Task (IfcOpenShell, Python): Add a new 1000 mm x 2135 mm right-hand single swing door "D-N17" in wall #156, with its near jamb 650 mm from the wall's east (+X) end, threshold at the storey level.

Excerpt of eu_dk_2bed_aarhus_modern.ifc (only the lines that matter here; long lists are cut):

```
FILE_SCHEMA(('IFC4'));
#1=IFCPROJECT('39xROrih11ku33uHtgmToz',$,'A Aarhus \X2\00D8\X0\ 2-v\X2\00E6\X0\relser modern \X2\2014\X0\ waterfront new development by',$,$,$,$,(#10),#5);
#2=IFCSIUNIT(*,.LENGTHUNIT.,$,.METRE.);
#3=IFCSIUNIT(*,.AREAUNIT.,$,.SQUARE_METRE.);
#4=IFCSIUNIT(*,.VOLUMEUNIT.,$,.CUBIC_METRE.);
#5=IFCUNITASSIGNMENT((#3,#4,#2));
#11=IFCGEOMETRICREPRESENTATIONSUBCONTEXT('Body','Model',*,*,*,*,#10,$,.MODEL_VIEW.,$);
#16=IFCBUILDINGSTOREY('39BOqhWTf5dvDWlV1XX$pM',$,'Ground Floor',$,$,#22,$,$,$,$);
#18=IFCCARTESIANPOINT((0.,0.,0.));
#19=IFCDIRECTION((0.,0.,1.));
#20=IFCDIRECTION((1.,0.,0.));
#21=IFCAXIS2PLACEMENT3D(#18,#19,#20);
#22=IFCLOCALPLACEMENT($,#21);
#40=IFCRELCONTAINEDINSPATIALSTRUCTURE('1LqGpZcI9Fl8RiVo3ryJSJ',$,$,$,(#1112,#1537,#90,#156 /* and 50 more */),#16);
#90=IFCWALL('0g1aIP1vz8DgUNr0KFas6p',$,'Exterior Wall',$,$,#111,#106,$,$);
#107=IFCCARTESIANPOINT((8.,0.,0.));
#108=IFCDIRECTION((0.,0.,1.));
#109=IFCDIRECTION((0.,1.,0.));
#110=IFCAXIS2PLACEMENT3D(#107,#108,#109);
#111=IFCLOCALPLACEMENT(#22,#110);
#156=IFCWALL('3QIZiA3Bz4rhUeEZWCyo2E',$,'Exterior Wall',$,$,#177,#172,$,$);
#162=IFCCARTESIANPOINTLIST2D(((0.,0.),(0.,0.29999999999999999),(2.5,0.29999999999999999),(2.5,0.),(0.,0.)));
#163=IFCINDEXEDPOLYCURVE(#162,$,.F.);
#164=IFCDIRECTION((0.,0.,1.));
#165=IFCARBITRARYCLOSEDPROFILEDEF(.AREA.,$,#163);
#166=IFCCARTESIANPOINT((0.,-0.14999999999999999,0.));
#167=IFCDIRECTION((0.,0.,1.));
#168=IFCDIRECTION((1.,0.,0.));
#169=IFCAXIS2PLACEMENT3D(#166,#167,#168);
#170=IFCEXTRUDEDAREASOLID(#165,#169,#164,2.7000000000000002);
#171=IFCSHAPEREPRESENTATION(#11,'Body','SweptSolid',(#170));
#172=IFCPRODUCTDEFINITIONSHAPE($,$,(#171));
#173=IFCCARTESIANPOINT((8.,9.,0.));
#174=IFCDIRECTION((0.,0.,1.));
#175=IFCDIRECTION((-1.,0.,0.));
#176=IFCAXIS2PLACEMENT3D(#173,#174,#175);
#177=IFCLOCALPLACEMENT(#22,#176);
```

```python
import numpy as np
import ifcopenshell
import ifcopenshell.api.feature
import ifcopenshell.api.geometry
import ifcopenshell.api.root
import ifcopenshell.api.spatial
import ifcopenshell.geom
import ifcopenshell.util.element
import ifcopenshell.util.placement
import ifcopenshell.util.representation
import ifcopenshell.util.shape
import ifcopenshell.util.unit

model = ifcopenshell.open("eu_dk_2bed_aarhus_modern.ifc")
unit_scale = ifcopenshell.util.unit.calculate_unit_scale(model)
settings = ifcopenshell.geom.settings()


def volume(element):
    """Net volume in cubic metres, openings subtracted."""
    shape = ifcopenshell.geom.create_shape(settings, element)
    return ifcopenshell.util.shape.get_volume(shape.geometry)


wall = model.by_id(156)
storey = ifcopenshell.util.element.get_container(wall, ifc_class="IfcBuildingStorey")
context = ifcopenshell.util.representation.get_context(model, "Model", "Body", "MODEL_VIEW")
before = volume(wall)

width, height, from_end, sill = 1, 2.135, 0.65, 0.0  # metres

# The wall runs along its own X axis, and the end named is its -X end.
wall_shape = ifcopenshell.geom.create_shape(settings, wall)
x, y, z = ifcopenshell.util.shape.get_vertices(wall_shape.geometry).T
start = x.min() + from_end
face, thickness = float(y.min()), float(y.max() - y.min())
wall_matrix = ifcopenshell.util.placement.get_local_placement(wall.ObjectPlacement)
level = ifcopenshell.util.placement.get_local_placement(storey.ObjectPlacement)[2, 3]


def in_wall(x, y):
    """Placement at x, y metres in the wall's axes, at sill height."""
    matrix = wall_matrix.copy()
    matrix[:, 3] = wall_matrix @ np.array([x / unit_scale, y / unit_scale, 0.0, 1.0])
    matrix[2, 3] = level + sill / unit_scale
    return matrix


# Opening: a box that overshoots both wall faces by 50 mm.
opening = ifcopenshell.api.root.create_entity(model, ifc_class="IfcOpeningElement", predefined_type="OPENING")
box = ifcopenshell.api.geometry.add_wall_representation(
    model, context=context, length=width, height=height, thickness=thickness + 0.1
)
ifcopenshell.api.geometry.assign_representation(model, product=opening, representation=box)
ifcopenshell.api.geometry.edit_object_placement(model, product=opening, matrix=in_wall(start, face - 0.05), is_si=False)
ifcopenshell.api.feature.add_feature(model, feature=opening, element=wall)

door = ifcopenshell.api.root.create_entity(model, ifc_class="IfcDoor", name="D-N17", predefined_type="DOOR")
door.OverallWidth, door.OverallHeight = width / unit_scale, height / unit_scale
door.OperationType = "SINGLE_SWING_RIGHT"
body = ifcopenshell.api.geometry.add_door_representation(
    model,
    context=context,
    overall_width=door.OverallWidth,
    overall_height=door.OverallHeight,
    operation_type="SINGLE_SWING_RIGHT",
    lining_properties={"LiningDepth": thickness / unit_scale, "ThresholdDepth": thickness / unit_scale},
)
ifcopenshell.api.geometry.assign_representation(model, product=door, representation=body)
ifcopenshell.api.spatial.assign_container(model, products=[door], relating_structure=storey)
ifcopenshell.api.feature.add_filling(model, opening=opening, element=door)

# The lining spans the wall, so the door starts at the wall face.
ifcopenshell.api.geometry.edit_object_placement(model, product=door, matrix=in_wall(start, face), is_si=False)

after = volume(wall)

print(f"wall volume {before:.3f} -> {after:.3f} m3")

model.write("eu_dk_2bed_aarhus_modern-out.ifc")
```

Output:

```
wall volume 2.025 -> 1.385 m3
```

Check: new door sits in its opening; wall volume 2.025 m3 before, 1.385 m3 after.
